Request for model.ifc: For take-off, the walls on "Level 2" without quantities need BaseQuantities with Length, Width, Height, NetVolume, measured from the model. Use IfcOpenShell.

First a look at what the model holds.

```python
import ifcopenshell
import ifcopenshell.util.element
import ifcopenshell.util.unit

model = ifcopenshell.open("model.ifc")
print(model.schema)
for unit_type in ("LENGTHUNIT", "AREAUNIT", "VOLUMEUNIT"):
    print(unit_type, ifcopenshell.util.unit.calculate_unit_scale(model, unit_type))
storey = next(s for s in model.by_type("IfcBuildingStorey") if s.Name == "Level 2")
walls = [e for e in ifcopenshell.util.element.get_decomposition(storey) if e.is_a("IfcWall")]
for e in sorted(walls, key=lambda e: e.id()):
    print(e.id(), e.is_a(), e.Name, list(ifcopenshell.util.element.get_psets(e, qtos_only=True)), sep=" | ")
```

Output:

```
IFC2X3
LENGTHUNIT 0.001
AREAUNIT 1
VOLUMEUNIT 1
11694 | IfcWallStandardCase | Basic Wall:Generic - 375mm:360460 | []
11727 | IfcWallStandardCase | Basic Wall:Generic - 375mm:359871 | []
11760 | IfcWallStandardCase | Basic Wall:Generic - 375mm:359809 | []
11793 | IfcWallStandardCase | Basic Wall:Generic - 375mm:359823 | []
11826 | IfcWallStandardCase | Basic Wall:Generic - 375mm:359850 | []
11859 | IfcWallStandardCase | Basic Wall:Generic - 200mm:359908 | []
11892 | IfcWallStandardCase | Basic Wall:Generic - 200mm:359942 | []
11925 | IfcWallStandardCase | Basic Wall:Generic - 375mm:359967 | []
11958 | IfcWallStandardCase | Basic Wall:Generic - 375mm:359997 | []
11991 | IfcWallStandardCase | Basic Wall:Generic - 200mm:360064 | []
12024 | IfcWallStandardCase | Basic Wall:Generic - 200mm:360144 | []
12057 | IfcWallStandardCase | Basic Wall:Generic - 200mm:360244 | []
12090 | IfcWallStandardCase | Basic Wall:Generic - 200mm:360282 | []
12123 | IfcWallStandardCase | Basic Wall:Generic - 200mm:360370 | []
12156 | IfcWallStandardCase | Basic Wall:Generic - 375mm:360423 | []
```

```python
import ifcopenshell
import ifcopenshell.api.pset
import ifcopenshell.geom
import ifcopenshell.util.element
import ifcopenshell.util.shape
import ifcopenshell.util.unit

model = ifcopenshell.open("model.ifc")
unit_scale = ifcopenshell.util.unit.calculate_unit_scale(model)
volume_scale = ifcopenshell.util.unit.calculate_unit_scale(model, "VOLUMEUNIT")
settings = ifcopenshell.geom.settings()

storey = next(s for s in model.by_type("IfcBuildingStorey") if s.Name == "Level 2")
walls = [e for e in ifcopenshell.util.element.get_decomposition(storey) if e.is_a("IfcWall")]

for e in sorted(walls, key=lambda e: e.id()):
    if ifcopenshell.util.element.get_psets(e, qtos_only=True, should_inherit=False):
        continue
    # Geometry comes back in metres, in the element's own axes.
    shape = ifcopenshell.geom.create_shape(settings, e)
    values = {
        "Length": ifcopenshell.util.shape.get_x(shape.geometry) / unit_scale,
        "Width": ifcopenshell.util.shape.get_y(shape.geometry) / unit_scale,
        "Height": ifcopenshell.util.shape.get_z(shape.geometry) / unit_scale,
        "NetVolume": ifcopenshell.util.shape.get_volume(shape.geometry) / volume_scale,
    }
    qto = ifcopenshell.api.pset.add_qto(model, product=e, name="BaseQuantities")
    ifcopenshell.api.pset.edit_qto(model, qto=qto, properties=values)
    print(e.id(), {k: round(v, 3) for k, v in values.items()})

model.write("model_v2.ifc")
```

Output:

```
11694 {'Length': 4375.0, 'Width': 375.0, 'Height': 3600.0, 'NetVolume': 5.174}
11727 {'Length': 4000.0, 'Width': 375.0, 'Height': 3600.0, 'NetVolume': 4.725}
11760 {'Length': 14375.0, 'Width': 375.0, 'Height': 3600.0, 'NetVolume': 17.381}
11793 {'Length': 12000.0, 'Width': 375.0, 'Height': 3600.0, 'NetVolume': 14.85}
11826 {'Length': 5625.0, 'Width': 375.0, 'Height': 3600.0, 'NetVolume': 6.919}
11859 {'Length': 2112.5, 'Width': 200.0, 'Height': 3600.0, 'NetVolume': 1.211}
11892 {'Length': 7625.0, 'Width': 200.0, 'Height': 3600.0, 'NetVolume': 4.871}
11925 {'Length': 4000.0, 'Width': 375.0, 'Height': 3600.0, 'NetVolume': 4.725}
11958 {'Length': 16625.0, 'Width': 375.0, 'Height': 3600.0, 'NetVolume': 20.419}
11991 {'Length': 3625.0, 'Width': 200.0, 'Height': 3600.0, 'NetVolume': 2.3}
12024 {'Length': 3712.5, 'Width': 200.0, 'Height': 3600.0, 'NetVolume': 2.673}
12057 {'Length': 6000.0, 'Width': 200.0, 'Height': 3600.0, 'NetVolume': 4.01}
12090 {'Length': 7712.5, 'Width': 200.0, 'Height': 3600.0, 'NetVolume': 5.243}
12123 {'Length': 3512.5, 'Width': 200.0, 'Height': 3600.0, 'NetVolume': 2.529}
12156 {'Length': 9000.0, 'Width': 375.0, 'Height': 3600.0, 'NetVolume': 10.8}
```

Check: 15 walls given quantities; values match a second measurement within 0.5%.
